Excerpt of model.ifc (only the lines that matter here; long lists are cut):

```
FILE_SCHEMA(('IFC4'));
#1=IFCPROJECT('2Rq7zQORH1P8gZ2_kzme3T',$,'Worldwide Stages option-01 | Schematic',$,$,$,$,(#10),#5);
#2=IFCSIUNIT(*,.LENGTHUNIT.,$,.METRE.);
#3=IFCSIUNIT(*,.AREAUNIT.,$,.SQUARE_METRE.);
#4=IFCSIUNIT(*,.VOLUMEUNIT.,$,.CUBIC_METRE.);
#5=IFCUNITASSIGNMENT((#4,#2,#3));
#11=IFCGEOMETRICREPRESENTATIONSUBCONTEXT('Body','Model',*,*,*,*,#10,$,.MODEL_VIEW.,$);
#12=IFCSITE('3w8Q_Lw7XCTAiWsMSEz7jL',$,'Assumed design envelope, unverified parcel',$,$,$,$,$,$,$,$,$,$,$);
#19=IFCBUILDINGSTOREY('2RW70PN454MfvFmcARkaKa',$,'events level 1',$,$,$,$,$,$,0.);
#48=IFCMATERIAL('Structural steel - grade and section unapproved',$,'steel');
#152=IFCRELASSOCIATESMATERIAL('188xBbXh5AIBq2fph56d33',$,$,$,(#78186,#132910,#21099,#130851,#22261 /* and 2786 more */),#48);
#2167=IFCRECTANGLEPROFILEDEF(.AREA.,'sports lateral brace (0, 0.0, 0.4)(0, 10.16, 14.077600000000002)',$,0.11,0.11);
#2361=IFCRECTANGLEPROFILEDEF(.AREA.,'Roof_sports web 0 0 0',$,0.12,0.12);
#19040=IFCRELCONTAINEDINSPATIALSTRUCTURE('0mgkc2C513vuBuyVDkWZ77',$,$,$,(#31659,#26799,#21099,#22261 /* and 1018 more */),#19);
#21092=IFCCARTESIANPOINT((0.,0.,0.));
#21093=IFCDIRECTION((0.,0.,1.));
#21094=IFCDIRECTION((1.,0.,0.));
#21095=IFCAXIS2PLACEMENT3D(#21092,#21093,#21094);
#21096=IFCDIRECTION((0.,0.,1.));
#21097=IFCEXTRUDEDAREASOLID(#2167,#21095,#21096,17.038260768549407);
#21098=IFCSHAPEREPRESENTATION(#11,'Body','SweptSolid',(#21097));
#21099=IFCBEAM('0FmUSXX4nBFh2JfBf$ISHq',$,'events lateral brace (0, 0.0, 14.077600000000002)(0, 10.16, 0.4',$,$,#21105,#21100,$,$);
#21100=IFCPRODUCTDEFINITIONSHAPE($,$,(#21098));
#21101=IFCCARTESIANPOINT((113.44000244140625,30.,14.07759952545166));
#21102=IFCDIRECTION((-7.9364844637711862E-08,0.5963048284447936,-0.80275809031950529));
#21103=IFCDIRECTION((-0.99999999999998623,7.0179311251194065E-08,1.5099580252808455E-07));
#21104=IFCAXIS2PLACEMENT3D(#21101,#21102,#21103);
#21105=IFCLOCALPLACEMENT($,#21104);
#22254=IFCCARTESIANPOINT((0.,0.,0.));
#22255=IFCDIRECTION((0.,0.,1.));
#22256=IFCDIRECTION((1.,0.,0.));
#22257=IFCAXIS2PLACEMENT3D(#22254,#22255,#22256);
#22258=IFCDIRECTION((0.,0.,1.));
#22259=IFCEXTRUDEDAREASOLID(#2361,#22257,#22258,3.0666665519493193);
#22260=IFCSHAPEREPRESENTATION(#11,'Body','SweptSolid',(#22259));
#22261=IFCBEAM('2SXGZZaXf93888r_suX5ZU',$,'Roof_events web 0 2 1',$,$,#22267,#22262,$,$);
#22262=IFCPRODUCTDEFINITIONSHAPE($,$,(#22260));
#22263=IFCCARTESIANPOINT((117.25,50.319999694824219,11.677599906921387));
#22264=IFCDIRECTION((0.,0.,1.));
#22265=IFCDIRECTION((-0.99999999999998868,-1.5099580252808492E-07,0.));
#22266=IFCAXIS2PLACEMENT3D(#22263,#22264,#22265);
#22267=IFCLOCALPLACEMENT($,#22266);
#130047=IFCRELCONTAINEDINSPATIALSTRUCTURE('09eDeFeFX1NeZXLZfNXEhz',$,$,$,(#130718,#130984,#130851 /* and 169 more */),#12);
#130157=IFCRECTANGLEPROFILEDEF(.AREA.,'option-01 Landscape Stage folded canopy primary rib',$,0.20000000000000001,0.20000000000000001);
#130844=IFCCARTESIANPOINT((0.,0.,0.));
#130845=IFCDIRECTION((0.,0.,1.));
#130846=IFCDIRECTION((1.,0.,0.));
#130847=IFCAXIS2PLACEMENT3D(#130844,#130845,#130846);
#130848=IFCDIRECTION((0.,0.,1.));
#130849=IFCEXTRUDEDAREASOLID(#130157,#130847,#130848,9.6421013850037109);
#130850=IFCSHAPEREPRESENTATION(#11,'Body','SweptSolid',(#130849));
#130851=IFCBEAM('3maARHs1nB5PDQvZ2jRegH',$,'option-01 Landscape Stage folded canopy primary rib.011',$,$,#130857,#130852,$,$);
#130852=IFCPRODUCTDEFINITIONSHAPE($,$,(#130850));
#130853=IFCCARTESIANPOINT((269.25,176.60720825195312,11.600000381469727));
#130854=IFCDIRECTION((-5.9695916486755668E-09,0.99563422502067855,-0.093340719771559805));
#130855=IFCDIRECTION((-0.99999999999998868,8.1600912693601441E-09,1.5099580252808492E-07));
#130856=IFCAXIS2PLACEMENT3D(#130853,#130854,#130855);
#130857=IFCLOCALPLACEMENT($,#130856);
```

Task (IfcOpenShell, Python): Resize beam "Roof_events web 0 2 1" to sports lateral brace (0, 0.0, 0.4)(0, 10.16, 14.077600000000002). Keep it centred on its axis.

```python
import ifcopenshell
import ifcopenshell.util.element
import ifcopenshell.util.representation

model = ifcopenshell.open("model.ifc")

member = model.by_guid("2SXGZZaXf93888r_suX5ZU")
source = next(p for p in model.by_type("IfcRectangleProfileDef") if p.ProfileName == "sports lateral brace (0, 0.0, 0.4)(0, 10.16, 14.077600000000002)")

body = ifcopenshell.util.representation.get_representation(member, "Model", "Body")
solid = body.Items[0]
old_profile = solid.SweptArea

# Copy the section's sizes but keep this member's own profile position.
profile = ifcopenshell.util.element.copy(model, source)
profile.Position = old_profile.Position
solid.SweptArea = profile
if not model.get_total_inverses(old_profile):
    ifcopenshell.util.element.remove_deep2(model, old_profile)

print(solid.SweptArea)

model.write("model-out.ifc")
```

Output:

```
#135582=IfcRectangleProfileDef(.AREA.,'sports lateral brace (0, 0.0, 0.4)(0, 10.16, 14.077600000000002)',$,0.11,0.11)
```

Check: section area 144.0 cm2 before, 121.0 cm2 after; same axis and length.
